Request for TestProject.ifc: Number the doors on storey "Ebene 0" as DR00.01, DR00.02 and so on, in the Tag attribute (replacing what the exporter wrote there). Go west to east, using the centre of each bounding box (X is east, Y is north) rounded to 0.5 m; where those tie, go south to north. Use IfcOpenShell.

First a look at what the model holds.

```python
import ifcopenshell
import ifcopenshell.util.element
import ifcopenshell.util.placement

model = ifcopenshell.open("TestProject.ifc")
print(model.schema)
storey = next(s for s in model.by_type("IfcBuildingStorey") if s.Name == "Ebene 0")
doors = [e for e in ifcopenshell.util.element.get_decomposition(storey) if e.is_a("IfcDoor")]
for e in sorted(doors, key=lambda e: e.id()):
    origin = ifcopenshell.util.placement.get_local_placement(e.ObjectPlacement)[:3, 3]
    print(e.id(), e.Tag, e.Name, origin.round(2) + 0.0, sep=" | ")
```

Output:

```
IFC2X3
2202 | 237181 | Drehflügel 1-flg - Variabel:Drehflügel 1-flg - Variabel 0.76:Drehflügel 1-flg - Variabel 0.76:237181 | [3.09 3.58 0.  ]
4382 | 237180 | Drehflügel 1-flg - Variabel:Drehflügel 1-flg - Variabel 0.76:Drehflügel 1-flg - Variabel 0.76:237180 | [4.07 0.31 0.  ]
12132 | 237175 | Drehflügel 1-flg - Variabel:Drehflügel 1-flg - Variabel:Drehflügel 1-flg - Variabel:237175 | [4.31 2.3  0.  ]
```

```python
import ifcopenshell
import ifcopenshell.geom
import ifcopenshell.util.element
import ifcopenshell.util.shape

model = ifcopenshell.open("TestProject.ifc")
settings = ifcopenshell.geom.settings()
settings.set("use-world-coords", True)


def centre(element):
    shape = ifcopenshell.geom.create_shape(settings, element)
    return ifcopenshell.util.shape.get_bbox_centroid(shape.geometry)


storey = next(s for s in model.by_type("IfcBuildingStorey") if s.Name == "Ebene 0")
doors = [e for e in ifcopenshell.util.element.get_decomposition(storey) if e.is_a("IfcDoor")]

# Insertion points can sit at a corner or the storey origin, so sort by the geometry (in metres).
centres = {e: centre(e) for e in doors}
doors.sort(key=lambda e: (round(centres[e][0] / 0.5), centres[e][1]))

for i, e in enumerate(doors, start=1):
    number = f"DR00.{i:02d}"
    e.Tag = number
    print(e.id(), number)

model.write("TestProject_rev.ifc")
```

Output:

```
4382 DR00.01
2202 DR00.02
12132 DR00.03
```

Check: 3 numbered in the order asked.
